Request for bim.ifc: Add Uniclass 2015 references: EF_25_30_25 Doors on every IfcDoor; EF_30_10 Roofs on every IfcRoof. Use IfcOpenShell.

First a look at what the model holds.

```python
import ifcopenshell

model = ifcopenshell.open("bim.ifc")
print(model.schema)
print("classifications:", [c.Name for c in model.by_type("IfcClassification")])
for ifc_class in ("IfcDoor", "IfcRoof", "IfcStair", "IfcWall", "IfcWindow"):
    print(ifc_class, len(model.by_type(ifc_class)))
```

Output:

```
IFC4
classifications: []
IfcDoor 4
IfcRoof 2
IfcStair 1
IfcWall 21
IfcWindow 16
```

```python
import ifcopenshell
import ifcopenshell.api.classification

model = ifcopenshell.open("bim.ifc")

system = ifcopenshell.api.classification.add_classification(model, classification="Uniclass 2015")

codes = {
    "IfcDoor": ("EF_25_30_25", "Doors"),
    "IfcRoof": ("EF_30_10", "Roofs"),
}
for ifc_class, (code, name) in codes.items():
    products = model.by_type(ifc_class)
    ifcopenshell.api.classification.add_reference(
        model, products=products, classification=system, identification=code, name=name
    )
    print(code, len(products))

model.write("bim-out.ifc")
```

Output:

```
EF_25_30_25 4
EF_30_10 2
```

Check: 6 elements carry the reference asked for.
